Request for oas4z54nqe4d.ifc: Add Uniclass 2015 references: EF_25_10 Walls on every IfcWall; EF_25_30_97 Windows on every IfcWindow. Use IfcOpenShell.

First a look at what the model holds.

```python
import ifcopenshell

model = ifcopenshell.open("oas4z54nqe4d.ifc")
print(model.schema)
print("classifications:", [c.Name for c in model.by_type("IfcClassification")])
for ifc_class in ("IfcDoor", "IfcRoof", "IfcStair", "IfcWall", "IfcWindow"):
    print(ifc_class, len(model.by_type(ifc_class)))
```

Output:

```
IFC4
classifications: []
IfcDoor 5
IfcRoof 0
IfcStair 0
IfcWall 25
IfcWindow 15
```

```python
import ifcopenshell
import ifcopenshell.api.classification

model = ifcopenshell.open("oas4z54nqe4d.ifc")

system = ifcopenshell.api.classification.add_classification(model, classification="Uniclass 2015")

codes = {
    "IfcWall": ("EF_25_10", "Walls"),
    "IfcWindow": ("EF_25_30_97", "Windows"),
}
for ifc_class, (code, name) in codes.items():
    products = model.by_type(ifc_class)
    ifcopenshell.api.classification.add_reference(
        model, products=products, classification=system, identification=code, name=name
    )
    print(code, len(products))

model.write("oas4z54nqe4d-out.ifc")
```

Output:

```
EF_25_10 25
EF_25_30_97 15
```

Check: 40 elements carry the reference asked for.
